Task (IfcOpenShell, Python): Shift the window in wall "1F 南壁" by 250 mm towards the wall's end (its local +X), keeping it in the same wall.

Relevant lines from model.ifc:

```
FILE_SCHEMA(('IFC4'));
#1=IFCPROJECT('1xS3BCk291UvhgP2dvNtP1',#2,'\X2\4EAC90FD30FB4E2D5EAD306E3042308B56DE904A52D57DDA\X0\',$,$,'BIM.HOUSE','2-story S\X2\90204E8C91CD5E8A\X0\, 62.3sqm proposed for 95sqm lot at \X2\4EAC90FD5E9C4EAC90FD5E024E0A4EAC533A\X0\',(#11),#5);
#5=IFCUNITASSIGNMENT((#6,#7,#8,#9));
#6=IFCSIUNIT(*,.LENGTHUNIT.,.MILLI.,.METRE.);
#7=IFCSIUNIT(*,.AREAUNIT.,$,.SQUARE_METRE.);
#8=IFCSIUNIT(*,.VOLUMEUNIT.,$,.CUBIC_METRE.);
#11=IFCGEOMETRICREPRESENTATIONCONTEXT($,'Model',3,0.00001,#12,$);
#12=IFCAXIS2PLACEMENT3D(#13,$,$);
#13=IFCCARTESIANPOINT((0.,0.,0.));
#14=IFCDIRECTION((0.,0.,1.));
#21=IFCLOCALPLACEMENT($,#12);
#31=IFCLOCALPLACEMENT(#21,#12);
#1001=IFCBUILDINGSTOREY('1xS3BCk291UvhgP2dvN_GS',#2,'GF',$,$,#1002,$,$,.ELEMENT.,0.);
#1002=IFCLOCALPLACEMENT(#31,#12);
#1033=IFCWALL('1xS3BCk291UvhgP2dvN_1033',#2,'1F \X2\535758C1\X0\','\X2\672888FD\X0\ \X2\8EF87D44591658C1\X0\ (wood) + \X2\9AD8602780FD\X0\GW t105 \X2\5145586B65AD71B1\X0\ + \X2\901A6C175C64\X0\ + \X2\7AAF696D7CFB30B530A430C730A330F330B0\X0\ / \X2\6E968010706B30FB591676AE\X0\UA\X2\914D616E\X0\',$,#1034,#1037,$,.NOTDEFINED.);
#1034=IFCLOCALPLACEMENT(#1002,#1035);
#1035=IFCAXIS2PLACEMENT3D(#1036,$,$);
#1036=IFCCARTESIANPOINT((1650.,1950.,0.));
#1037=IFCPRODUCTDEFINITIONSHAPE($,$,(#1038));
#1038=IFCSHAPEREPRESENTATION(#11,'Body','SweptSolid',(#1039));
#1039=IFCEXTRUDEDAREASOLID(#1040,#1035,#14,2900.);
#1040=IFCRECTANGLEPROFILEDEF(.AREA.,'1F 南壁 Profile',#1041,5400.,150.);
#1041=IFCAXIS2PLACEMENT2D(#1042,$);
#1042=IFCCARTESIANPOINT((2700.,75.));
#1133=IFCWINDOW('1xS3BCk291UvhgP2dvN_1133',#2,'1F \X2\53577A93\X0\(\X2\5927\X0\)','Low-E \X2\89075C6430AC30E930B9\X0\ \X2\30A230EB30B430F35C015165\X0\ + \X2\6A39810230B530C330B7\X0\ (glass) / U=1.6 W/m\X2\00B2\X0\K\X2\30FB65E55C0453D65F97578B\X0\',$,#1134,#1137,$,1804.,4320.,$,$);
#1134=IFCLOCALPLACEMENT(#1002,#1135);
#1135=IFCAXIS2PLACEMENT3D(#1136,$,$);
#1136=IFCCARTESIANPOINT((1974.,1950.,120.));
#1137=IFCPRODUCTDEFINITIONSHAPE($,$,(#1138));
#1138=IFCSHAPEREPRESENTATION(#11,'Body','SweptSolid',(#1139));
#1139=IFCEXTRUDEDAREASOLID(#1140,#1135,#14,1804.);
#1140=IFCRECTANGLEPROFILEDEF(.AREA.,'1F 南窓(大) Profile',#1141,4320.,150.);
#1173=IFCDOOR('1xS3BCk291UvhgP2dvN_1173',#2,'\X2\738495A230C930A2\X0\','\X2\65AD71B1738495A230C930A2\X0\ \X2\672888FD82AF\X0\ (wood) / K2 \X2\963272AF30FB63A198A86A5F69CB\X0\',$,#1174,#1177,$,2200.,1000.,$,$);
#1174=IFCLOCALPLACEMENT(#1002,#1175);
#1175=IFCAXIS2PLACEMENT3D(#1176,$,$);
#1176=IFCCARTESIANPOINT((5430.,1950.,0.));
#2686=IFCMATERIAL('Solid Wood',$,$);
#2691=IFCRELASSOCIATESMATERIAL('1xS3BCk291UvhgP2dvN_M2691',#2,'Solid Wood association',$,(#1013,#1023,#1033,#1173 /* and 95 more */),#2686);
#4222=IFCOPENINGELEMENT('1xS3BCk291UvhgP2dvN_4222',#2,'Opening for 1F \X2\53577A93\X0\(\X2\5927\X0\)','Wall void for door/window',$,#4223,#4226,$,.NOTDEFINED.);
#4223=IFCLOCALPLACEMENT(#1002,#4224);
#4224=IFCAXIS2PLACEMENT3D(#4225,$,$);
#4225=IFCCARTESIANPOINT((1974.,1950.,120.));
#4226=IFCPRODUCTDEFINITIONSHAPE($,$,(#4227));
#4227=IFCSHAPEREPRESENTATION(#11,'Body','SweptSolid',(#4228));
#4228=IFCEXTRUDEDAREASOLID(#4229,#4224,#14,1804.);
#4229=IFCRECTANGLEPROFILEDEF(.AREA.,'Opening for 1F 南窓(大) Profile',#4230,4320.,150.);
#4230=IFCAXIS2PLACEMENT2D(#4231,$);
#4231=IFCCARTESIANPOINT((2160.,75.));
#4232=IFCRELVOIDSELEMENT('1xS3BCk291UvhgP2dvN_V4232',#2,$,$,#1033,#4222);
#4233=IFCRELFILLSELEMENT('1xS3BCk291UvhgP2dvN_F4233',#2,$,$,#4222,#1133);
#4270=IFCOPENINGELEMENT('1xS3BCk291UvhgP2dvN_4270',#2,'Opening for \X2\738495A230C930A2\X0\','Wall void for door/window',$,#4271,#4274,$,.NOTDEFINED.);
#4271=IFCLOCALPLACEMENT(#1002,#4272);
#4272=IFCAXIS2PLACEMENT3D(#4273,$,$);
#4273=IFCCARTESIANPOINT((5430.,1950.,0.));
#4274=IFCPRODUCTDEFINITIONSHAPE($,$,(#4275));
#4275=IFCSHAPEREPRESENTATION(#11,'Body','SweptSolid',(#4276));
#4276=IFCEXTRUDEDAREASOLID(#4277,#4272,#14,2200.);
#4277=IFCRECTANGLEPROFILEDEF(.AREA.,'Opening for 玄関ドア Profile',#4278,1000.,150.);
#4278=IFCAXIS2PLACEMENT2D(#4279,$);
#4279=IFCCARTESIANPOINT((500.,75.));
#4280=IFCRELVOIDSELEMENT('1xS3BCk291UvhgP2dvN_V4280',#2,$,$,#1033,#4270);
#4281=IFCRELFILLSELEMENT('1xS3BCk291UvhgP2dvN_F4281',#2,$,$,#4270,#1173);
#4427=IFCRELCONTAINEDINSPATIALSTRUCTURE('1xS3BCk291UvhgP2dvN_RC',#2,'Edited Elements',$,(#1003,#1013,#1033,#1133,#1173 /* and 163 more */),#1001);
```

```python
import ifcopenshell
import ifcopenshell.api.geometry
import ifcopenshell.util.placement

model = ifcopenshell.open("model.ifc")

window = model.by_guid("1xS3BCk291UvhgP2dvN_1133")
opening = window.FillsVoids[0].RelatingOpeningElement
wall = opening.VoidsElements[0].RelatingBuildingElement

wall_matrix = ifcopenshell.util.placement.get_local_placement(wall.ObjectPlacement)
shift = wall_matrix[:3, 0] * 250.0
before = ifcopenshell.util.placement.get_local_placement(window.ObjectPlacement)[:3, 3].copy()

# The window is not placed relative to its opening, so move both.
for product in (opening, window):
    matrix = ifcopenshell.util.placement.get_local_placement(product.ObjectPlacement)
    matrix[:3, 3] += shift
    ifcopenshell.api.geometry.edit_object_placement(model, product=product, matrix=matrix, is_si=False)

after = ifcopenshell.util.placement.get_local_placement(window.ObjectPlacement)[:3, 3]
print("window moved by", (after - before).round(3) + 0.0)

model.write("model-out.ifc")
```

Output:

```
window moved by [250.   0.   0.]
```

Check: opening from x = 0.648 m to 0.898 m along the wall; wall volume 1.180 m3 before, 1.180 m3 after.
